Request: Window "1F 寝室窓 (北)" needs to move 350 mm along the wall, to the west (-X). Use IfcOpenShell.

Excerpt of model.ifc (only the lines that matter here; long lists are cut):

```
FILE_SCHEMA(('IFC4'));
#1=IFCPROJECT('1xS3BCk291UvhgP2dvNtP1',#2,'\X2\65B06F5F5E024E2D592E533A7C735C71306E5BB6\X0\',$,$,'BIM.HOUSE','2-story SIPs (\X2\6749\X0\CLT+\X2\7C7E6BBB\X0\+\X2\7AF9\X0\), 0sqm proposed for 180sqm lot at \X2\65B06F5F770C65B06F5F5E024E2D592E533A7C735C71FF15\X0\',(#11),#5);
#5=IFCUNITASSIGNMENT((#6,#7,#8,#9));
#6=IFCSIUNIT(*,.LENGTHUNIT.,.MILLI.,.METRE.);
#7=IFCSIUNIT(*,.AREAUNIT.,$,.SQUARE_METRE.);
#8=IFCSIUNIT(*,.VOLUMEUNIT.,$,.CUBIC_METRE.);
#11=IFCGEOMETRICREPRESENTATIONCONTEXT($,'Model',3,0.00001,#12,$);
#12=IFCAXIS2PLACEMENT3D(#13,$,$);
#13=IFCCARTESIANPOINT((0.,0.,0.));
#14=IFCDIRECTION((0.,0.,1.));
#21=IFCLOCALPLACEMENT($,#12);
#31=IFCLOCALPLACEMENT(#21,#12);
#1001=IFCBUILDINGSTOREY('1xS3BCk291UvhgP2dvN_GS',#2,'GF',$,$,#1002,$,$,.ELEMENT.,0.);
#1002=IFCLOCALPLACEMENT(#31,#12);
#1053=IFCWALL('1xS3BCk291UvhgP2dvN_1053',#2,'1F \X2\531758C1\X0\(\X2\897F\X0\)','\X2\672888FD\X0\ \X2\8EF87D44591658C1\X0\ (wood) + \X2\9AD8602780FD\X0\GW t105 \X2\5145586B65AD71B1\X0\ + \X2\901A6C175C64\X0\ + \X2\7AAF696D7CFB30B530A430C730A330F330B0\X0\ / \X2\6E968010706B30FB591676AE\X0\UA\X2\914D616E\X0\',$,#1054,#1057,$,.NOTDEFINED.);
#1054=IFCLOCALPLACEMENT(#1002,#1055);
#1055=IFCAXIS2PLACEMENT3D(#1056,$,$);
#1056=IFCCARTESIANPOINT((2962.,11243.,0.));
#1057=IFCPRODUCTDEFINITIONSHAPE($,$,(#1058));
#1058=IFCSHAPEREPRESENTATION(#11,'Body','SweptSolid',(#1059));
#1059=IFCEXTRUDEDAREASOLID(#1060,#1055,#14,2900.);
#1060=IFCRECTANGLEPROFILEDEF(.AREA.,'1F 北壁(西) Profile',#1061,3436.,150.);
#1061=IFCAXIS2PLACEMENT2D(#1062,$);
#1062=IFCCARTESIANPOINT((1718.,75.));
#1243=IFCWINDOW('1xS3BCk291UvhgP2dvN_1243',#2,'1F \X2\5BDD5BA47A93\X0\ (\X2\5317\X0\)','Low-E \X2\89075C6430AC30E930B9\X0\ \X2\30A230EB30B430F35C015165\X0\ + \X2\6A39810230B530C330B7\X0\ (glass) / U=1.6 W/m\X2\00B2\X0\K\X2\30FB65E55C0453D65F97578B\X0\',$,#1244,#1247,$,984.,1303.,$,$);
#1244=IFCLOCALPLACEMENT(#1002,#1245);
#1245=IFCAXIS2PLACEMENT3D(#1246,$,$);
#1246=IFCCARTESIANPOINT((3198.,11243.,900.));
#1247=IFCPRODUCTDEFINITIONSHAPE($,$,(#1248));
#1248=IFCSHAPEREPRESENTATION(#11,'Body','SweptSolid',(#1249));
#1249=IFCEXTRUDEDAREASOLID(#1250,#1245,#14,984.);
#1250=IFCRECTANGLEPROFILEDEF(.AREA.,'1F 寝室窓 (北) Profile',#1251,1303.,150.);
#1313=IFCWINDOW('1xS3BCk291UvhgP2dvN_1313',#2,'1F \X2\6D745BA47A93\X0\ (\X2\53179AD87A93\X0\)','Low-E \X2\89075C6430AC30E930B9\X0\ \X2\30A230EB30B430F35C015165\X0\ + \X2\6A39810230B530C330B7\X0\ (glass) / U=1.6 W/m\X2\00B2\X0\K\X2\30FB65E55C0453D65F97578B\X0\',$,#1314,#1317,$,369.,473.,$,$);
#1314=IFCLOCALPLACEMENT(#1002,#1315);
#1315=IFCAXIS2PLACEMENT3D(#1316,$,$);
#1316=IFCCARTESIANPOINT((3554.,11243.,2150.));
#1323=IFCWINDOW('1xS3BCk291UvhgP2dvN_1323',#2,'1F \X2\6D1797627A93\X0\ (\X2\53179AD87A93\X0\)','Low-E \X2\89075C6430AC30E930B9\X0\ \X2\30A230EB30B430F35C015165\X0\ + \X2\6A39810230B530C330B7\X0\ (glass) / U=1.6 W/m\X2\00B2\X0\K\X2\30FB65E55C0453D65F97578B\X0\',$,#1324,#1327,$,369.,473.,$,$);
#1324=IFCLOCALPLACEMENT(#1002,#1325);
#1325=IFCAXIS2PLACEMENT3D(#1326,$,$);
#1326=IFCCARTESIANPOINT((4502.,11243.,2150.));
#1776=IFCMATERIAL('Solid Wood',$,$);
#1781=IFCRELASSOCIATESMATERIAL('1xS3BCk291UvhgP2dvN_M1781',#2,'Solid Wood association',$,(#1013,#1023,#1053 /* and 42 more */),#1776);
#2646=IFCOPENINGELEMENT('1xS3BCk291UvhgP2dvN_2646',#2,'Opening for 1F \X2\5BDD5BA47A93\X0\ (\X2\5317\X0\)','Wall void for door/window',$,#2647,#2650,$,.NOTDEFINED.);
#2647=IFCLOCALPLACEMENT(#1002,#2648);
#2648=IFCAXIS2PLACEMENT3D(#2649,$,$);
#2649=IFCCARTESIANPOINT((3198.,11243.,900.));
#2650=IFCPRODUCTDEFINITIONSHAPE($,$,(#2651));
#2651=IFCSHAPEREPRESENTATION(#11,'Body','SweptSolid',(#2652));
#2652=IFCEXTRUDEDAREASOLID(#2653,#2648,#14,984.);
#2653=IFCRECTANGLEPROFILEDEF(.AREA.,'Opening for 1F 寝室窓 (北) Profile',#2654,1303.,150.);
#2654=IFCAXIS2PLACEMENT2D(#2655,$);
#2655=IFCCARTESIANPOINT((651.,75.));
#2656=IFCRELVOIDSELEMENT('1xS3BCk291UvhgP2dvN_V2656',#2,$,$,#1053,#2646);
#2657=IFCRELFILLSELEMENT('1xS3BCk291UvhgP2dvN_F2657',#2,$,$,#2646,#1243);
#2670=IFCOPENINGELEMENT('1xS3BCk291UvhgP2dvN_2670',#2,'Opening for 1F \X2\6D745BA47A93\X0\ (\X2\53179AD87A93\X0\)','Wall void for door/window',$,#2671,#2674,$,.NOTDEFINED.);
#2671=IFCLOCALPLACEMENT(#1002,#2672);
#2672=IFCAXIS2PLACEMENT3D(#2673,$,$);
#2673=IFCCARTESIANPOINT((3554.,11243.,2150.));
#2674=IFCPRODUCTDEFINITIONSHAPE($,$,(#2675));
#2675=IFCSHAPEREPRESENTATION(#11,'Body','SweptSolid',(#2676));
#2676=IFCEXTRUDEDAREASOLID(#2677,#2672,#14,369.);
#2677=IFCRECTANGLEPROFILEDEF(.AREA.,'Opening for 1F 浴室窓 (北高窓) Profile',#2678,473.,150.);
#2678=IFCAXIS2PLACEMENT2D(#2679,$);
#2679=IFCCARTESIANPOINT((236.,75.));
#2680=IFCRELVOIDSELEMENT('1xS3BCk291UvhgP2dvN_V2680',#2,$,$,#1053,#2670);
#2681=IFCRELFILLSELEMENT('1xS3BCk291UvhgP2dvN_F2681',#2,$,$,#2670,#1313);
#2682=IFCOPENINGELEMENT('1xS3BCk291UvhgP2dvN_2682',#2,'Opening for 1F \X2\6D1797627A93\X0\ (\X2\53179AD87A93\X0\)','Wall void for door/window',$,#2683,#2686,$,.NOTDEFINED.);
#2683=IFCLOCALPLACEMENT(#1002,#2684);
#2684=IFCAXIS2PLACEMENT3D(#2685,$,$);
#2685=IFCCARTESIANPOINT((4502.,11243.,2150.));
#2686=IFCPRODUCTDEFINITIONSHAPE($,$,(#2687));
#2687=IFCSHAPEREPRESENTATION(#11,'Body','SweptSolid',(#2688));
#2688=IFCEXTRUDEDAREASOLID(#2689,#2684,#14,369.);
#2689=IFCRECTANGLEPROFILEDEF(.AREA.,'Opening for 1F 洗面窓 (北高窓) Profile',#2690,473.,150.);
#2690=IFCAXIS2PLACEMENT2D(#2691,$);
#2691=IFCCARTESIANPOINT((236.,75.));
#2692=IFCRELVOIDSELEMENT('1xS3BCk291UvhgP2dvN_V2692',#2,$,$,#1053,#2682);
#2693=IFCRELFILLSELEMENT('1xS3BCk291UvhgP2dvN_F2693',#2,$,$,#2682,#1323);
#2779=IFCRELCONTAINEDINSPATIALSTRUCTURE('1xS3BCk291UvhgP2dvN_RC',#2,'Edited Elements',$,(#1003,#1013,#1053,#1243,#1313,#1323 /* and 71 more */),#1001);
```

```python
import ifcopenshell
import ifcopenshell.api.geometry
import ifcopenshell.util.placement
import ifcopenshell.util.unit

model = ifcopenshell.open("model.ifc")
unit_scale = ifcopenshell.util.unit.calculate_unit_scale(model)

window = model.by_id(1243)
opening = window.FillsVoids[0].RelatingOpeningElement
wall = opening.VoidsElements[0].RelatingBuildingElement

wall_matrix = ifcopenshell.util.placement.get_local_placement(wall.ObjectPlacement)
shift = wall_matrix[:3, 0] * -0.35 / unit_scale
before = ifcopenshell.util.placement.get_local_placement(window.ObjectPlacement)[:3, 3].copy()

# The window is not placed relative to its opening, so move both.
for product in (opening, window):
    matrix = ifcopenshell.util.placement.get_local_placement(product.ObjectPlacement)
    matrix[:3, 3] += shift
    ifcopenshell.api.geometry.edit_object_placement(model, product=product, matrix=matrix, is_si=False)

after = ifcopenshell.util.placement.get_local_placement(window.ObjectPlacement)[:3, 3]
print("window moved by", (after - before).round(3) + 0.0)

model.write("model-out.ifc")
```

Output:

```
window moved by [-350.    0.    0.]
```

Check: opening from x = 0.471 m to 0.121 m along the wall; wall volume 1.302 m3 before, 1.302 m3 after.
